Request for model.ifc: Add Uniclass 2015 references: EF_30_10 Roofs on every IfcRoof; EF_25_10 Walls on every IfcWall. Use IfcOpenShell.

First a look at what the model holds.

```python
import ifcopenshell

model = ifcopenshell.open("model.ifc")
print(model.schema)
print("classifications:", [c.Name for c in model.by_type("IfcClassification")])
for ifc_class in ("IfcDoor", "IfcRoof", "IfcStair", "IfcWall", "IfcWindow"):
    print(ifc_class, len(model.by_type(ifc_class)))
```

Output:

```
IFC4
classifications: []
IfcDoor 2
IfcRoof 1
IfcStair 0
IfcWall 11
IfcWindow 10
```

```python
import ifcopenshell
import ifcopenshell.api.classification

model = ifcopenshell.open("model.ifc")

system = ifcopenshell.api.classification.add_classification(model, classification="Uniclass 2015")

codes = {
    "IfcRoof": ("EF_30_10", "Roofs"),
    "IfcWall": ("EF_25_10", "Walls"),
}
for ifc_class, (code, name) in codes.items():
    products = model.by_type(ifc_class)
    ifcopenshell.api.classification.add_reference(
        model, products=products, classification=system, identification=code, name=name
    )
    print(code, len(products))

model.write("model_edited.ifc")
```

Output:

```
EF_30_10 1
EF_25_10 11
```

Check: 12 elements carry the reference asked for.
